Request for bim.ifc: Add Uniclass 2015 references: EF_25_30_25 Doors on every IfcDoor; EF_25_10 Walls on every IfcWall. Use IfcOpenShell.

First a look at what the model holds.

```python
import ifcopenshell

model = ifcopenshell.open("bim.ifc")
print(model.schema)
print("classifications:", [c.Name for c in model.by_type("IfcClassification")])
for ifc_class in ("IfcDoor", "IfcRoof", "IfcStair", "IfcWall", "IfcWindow"):
    print(ifc_class, len(model.by_type(ifc_class)))
```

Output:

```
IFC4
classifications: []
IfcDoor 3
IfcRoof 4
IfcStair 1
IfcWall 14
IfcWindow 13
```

```python
import ifcopenshell
import ifcopenshell.api.classification

model = ifcopenshell.open("bim.ifc")

system = ifcopenshell.api.classification.add_classification(model, classification="Uniclass 2015")

codes = {
    "IfcDoor": ("EF_25_30_25", "Doors"),
    "IfcWall": ("EF_25_10", "Walls"),
}
for ifc_class, (code, name) in codes.items():
    products = model.by_type(ifc_class)
    ifcopenshell.api.classification.add_reference(
        model, products=products, classification=system, identification=code, name=name
    )
    print(code, len(products))

model.write("bim_rev.ifc")
```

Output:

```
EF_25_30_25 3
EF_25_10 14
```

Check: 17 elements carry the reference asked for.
